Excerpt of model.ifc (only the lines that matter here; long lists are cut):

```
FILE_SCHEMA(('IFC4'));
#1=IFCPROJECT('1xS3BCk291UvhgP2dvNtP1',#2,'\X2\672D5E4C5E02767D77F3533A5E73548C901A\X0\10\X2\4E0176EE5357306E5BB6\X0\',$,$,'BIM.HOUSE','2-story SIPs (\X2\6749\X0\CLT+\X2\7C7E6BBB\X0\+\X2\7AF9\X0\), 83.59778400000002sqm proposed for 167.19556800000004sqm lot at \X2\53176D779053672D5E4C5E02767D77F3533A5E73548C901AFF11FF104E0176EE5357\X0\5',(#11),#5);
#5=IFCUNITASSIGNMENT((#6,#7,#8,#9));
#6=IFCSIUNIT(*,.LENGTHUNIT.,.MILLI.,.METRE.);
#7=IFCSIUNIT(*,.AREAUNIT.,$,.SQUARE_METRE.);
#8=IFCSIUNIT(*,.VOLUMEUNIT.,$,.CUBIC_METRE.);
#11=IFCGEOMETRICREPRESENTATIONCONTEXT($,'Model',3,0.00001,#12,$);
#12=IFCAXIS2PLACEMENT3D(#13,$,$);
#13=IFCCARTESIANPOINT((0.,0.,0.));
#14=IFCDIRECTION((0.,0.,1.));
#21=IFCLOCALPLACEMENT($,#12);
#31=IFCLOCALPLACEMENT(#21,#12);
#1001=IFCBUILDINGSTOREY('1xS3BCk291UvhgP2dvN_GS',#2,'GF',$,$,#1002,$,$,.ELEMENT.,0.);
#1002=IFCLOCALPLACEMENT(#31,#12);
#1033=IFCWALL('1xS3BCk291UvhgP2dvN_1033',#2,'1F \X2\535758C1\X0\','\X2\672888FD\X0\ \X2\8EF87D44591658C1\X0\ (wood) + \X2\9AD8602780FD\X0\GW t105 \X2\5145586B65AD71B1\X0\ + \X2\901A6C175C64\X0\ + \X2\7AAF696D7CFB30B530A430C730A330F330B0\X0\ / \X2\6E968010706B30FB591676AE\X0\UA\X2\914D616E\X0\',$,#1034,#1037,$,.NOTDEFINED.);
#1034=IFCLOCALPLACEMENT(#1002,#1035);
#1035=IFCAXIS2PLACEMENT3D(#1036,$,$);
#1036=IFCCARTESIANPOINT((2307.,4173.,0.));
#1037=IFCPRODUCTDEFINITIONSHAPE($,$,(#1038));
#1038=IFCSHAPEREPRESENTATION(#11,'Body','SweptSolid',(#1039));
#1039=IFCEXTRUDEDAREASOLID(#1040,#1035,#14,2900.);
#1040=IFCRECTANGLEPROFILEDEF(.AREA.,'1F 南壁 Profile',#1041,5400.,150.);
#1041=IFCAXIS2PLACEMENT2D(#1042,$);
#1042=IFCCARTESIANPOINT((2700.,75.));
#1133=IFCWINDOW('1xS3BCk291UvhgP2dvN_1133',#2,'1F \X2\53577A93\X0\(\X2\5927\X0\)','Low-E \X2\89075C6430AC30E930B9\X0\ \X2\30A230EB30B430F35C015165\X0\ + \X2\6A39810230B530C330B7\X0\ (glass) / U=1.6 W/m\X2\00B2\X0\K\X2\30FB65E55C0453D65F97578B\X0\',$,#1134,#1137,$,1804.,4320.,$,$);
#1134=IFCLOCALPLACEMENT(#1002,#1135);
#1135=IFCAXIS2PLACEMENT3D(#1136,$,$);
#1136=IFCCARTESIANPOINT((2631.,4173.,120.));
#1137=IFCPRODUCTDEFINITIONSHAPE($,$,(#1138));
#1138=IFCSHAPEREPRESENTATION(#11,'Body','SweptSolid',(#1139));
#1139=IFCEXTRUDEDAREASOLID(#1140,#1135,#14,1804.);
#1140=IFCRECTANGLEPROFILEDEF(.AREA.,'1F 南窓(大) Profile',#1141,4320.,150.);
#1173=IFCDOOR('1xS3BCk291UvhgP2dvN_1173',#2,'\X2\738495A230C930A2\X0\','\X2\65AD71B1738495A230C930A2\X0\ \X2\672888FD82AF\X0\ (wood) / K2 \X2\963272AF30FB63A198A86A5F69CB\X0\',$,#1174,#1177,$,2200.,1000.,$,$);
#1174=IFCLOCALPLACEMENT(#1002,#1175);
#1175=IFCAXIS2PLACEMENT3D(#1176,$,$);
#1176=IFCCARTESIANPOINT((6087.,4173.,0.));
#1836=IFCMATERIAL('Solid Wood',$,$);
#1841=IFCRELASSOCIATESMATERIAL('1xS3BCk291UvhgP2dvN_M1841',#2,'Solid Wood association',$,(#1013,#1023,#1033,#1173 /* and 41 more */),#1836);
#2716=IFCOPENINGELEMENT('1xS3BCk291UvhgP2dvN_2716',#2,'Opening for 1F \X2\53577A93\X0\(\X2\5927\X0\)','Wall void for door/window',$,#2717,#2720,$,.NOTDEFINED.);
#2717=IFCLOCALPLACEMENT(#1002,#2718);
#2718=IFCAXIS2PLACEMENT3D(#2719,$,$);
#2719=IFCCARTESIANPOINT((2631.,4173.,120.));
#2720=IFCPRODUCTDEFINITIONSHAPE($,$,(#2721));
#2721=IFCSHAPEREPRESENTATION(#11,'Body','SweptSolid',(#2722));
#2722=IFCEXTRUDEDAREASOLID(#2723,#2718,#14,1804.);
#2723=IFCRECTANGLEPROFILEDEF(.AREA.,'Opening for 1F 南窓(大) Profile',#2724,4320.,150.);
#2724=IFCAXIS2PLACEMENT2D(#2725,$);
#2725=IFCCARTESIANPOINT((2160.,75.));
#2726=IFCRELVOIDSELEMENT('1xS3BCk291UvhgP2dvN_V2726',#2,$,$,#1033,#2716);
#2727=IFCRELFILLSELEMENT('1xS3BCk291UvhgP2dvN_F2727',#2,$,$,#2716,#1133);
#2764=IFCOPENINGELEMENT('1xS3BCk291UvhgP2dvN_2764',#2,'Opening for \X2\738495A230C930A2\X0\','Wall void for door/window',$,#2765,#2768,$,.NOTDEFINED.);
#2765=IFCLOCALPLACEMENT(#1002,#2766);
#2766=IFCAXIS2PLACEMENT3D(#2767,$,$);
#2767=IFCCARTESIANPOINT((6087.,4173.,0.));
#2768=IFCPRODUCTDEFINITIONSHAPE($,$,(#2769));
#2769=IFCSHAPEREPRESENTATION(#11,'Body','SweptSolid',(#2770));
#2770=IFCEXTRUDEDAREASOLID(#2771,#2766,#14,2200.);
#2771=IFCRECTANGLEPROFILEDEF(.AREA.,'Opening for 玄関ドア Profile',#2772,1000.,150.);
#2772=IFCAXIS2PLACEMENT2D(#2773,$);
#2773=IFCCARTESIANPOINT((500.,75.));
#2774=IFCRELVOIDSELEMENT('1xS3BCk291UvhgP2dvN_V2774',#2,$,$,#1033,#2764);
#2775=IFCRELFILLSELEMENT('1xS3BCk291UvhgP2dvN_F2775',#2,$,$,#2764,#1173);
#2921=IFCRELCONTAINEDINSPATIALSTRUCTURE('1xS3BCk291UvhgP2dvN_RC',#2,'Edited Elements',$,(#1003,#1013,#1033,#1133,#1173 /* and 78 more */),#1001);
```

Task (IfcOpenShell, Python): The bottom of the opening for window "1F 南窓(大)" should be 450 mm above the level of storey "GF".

```python
import numpy as np
import ifcopenshell
import ifcopenshell.api.geometry
import ifcopenshell.geom
import ifcopenshell.util.element
import ifcopenshell.util.placement
import ifcopenshell.util.shape
import ifcopenshell.util.unit

model = ifcopenshell.open("model.ifc")
unit_scale = ifcopenshell.util.unit.calculate_unit_scale(model)

window = model.by_guid("1xS3BCk291UvhgP2dvN_1133")
opening = window.FillsVoids[0].RelatingOpeningElement
storey = ifcopenshell.util.element.get_container(window, ifc_class="IfcBuildingStorey")
level = ifcopenshell.util.placement.get_local_placement(storey.ObjectPlacement)[2, 3]

# The opening's origin need not be at the sill, so measure its lowest point.
shape = ifcopenshell.geom.create_shape(ifcopenshell.geom.settings(), opening)
bottom = ifcopenshell.util.shape.get_shape_bottom_elevation(shape, shape.geometry) / unit_scale
dz = level + 450.0 - bottom

shift = np.array([0.0, 0.0, dz])
# The window is not placed relative to its opening, so move both.
for product in (opening, window):
    matrix = ifcopenshell.util.placement.get_local_placement(product.ObjectPlacement)
    matrix[:3, 3] += shift
    ifcopenshell.api.geometry.edit_object_placement(model, product=product, matrix=matrix, is_si=False)

print(f"moved by {dz * unit_scale:+.3f} m")

model.write("model_rev.ifc")
```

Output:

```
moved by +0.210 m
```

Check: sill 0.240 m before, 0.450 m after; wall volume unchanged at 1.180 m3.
